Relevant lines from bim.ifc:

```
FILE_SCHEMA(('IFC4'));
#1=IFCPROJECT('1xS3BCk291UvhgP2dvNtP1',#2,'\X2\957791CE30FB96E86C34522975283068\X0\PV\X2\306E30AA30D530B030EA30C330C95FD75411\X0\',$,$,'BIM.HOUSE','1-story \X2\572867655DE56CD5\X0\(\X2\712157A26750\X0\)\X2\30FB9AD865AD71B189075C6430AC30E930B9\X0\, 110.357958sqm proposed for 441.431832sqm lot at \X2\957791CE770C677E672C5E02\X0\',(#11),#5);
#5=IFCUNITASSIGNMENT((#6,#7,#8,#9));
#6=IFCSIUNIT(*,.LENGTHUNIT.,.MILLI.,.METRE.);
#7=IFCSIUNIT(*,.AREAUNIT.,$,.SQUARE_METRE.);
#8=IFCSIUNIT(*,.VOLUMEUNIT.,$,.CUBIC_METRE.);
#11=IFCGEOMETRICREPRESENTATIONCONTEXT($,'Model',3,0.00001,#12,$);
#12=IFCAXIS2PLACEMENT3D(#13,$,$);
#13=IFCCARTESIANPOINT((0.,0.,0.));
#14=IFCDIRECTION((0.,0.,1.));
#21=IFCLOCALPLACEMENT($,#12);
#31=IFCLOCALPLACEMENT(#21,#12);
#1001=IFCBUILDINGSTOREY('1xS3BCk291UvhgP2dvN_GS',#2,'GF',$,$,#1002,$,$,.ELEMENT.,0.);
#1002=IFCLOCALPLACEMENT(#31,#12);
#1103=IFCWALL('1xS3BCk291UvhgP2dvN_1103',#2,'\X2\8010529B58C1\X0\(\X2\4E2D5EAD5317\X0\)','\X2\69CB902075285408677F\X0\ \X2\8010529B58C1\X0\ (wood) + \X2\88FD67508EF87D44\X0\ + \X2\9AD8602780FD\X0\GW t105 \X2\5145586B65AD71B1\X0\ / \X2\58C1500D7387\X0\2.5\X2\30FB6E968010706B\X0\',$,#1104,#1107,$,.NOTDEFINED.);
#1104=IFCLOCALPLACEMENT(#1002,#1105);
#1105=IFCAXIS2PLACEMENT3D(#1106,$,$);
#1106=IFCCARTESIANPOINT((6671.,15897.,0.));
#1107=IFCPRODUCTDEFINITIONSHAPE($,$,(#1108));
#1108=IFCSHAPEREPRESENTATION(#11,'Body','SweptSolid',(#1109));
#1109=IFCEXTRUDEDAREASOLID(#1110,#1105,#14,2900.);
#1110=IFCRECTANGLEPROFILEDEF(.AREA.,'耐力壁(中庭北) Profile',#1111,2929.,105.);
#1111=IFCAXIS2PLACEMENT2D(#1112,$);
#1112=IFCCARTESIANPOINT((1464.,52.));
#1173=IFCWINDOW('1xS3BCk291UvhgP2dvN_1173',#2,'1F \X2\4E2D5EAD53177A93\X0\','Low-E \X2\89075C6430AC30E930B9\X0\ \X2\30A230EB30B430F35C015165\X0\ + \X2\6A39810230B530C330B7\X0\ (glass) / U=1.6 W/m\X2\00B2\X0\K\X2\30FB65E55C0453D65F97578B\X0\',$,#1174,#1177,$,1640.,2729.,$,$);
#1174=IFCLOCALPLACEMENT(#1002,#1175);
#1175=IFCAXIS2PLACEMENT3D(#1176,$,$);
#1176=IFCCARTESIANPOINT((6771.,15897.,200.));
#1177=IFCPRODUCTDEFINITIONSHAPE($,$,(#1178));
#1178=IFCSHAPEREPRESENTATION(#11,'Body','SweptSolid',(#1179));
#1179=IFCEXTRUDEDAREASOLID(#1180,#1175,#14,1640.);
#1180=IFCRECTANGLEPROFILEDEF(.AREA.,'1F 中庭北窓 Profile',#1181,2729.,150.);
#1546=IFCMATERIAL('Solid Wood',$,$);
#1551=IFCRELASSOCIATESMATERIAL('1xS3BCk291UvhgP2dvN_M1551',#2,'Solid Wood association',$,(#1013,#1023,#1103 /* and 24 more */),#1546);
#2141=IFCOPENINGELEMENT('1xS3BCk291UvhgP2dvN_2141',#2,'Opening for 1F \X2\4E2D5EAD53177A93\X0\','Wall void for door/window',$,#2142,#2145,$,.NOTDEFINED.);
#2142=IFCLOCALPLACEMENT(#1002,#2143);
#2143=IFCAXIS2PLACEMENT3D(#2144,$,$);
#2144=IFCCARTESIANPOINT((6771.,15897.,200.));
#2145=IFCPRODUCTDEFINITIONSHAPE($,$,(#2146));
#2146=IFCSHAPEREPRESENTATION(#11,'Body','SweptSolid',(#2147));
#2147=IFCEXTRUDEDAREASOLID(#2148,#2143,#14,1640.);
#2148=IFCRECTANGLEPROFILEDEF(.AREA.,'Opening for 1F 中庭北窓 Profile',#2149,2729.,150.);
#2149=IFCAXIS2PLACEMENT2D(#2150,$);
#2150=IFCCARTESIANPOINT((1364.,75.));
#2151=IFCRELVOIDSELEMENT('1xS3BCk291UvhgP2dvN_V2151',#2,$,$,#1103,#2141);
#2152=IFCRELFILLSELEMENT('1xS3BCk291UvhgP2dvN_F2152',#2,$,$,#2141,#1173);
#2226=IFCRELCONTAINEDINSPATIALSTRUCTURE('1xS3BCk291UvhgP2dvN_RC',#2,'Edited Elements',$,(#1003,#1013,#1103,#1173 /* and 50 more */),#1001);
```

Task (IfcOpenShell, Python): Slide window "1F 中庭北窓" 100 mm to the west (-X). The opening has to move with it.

```python
import ifcopenshell
import ifcopenshell.api.geometry
import ifcopenshell.util.placement
import ifcopenshell.util.unit

model = ifcopenshell.open("bim.ifc")
unit_scale = ifcopenshell.util.unit.calculate_unit_scale(model)

window = model.by_guid("1xS3BCk291UvhgP2dvN_1173")
opening = window.FillsVoids[0].RelatingOpeningElement
wall = opening.VoidsElements[0].RelatingBuildingElement

wall_matrix = ifcopenshell.util.placement.get_local_placement(wall.ObjectPlacement)
shift = wall_matrix[:3, 0] * -0.1 / unit_scale
before = ifcopenshell.util.placement.get_local_placement(window.ObjectPlacement)[:3, 3].copy()

# The window is not placed relative to its opening, so move both.
for product in (opening, window):
    matrix = ifcopenshell.util.placement.get_local_placement(product.ObjectPlacement)
    matrix[:3, 3] += shift
    ifcopenshell.api.geometry.edit_object_placement(model, product=product, matrix=matrix, is_si=False)

after = ifcopenshell.util.placement.get_local_placement(window.ObjectPlacement)[:3, 3]
print("window moved by", (after - before).round(3) + 0.0)

model.write("bim_updated.ifc")
```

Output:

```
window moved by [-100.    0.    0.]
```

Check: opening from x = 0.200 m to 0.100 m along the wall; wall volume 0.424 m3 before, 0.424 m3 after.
